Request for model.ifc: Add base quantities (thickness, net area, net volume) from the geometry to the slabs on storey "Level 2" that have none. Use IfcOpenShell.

First a look at what the model holds.

```python
import ifcopenshell
import ifcopenshell.util.element
import ifcopenshell.util.unit

model = ifcopenshell.open("model.ifc")
print(model.schema)
for unit_type in ("LENGTHUNIT", "AREAUNIT", "VOLUMEUNIT"):
    print(unit_type, ifcopenshell.util.unit.calculate_unit_scale(model, unit_type))
storey = next(s for s in model.by_type("IfcBuildingStorey") if s.Name == "Level 2")
slabs = [e for e in ifcopenshell.util.element.get_decomposition(storey) if e.is_a("IfcSlab")]
for e in sorted(slabs, key=lambda e: e.id()):
    print(e.id(), e.is_a(), e.Name, list(ifcopenshell.util.element.get_psets(e, qtos_only=True)), sep=" | ")
```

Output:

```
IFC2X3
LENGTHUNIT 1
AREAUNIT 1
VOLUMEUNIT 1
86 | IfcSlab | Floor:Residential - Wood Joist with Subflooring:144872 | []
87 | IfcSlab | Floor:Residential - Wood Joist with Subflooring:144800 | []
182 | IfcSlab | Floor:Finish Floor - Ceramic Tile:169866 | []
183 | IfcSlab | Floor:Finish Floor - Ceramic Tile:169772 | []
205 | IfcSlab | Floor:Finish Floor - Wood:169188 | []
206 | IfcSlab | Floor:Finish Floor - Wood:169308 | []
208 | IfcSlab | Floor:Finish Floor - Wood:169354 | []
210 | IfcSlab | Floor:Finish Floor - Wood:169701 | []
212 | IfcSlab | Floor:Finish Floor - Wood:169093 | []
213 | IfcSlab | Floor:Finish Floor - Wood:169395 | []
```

```python
import ifcopenshell
import ifcopenshell.api.pset
import ifcopenshell.geom
import ifcopenshell.util.element
import ifcopenshell.util.shape
import ifcopenshell.util.unit

model = ifcopenshell.open("model.ifc")
unit_scale = ifcopenshell.util.unit.calculate_unit_scale(model)
area_scale = ifcopenshell.util.unit.calculate_unit_scale(model, "AREAUNIT")
volume_scale = ifcopenshell.util.unit.calculate_unit_scale(model, "VOLUMEUNIT")
settings = ifcopenshell.geom.settings()

storey = next(s for s in model.by_type("IfcBuildingStorey") if s.Name == "Level 2")
slabs = [e for e in ifcopenshell.util.element.get_decomposition(storey) if e.is_a("IfcSlab")]

for e in sorted(slabs, key=lambda e: e.id()):
    if ifcopenshell.util.element.get_psets(e, qtos_only=True, should_inherit=False):
        continue
    # Geometry comes back in metres, in the element's own axes.
    shape = ifcopenshell.geom.create_shape(settings, e)
    values = {
        "Width": ifcopenshell.util.shape.get_z(shape.geometry) / unit_scale,
        "NetArea": ifcopenshell.util.shape.get_footprint_area(shape.geometry) / area_scale,
        "NetVolume": ifcopenshell.util.shape.get_volume(shape.geometry) / volume_scale,
    }
    qto = ifcopenshell.api.pset.add_qto(model, product=e, name="BaseQuantities")
    ifcopenshell.api.pset.edit_qto(model, qto=qto, properties=values)
    print(e.id(), {k: round(v, 3) for k, v in values.items()})

model.write("model_v2.ifc")
```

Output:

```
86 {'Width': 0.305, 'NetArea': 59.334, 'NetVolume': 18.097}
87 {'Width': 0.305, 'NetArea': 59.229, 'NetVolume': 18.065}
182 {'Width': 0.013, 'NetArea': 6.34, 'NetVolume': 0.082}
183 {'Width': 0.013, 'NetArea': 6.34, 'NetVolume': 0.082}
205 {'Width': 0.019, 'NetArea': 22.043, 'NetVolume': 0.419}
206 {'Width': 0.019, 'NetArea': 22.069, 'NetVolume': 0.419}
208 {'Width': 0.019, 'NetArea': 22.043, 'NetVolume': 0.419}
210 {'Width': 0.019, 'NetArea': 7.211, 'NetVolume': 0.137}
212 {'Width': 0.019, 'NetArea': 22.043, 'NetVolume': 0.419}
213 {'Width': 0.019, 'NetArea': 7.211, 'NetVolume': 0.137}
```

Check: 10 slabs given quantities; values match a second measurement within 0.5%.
